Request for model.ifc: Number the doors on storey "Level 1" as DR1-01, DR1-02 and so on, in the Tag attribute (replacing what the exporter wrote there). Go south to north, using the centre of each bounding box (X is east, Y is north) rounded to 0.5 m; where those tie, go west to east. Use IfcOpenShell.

First a look at what the model holds.

```python
import ifcopenshell
import ifcopenshell.util.element
import ifcopenshell.util.placement

model = ifcopenshell.open("model.ifc")
print(model.schema)
storey = next(s for s in model.by_type("IfcBuildingStorey") if s.Name == "Level 1")
doors = [e for e in ifcopenshell.util.element.get_decomposition(storey) if e.is_a("IfcDoor")]
for e in sorted(doors, key=lambda e: e.id()):
    origin = ifcopenshell.util.placement.get_local_placement(e.ObjectPlacement)[:3, 3]
    print(e.id(), e.Tag, e.Name, origin.round(2) + 0.0, sep=" | ")
```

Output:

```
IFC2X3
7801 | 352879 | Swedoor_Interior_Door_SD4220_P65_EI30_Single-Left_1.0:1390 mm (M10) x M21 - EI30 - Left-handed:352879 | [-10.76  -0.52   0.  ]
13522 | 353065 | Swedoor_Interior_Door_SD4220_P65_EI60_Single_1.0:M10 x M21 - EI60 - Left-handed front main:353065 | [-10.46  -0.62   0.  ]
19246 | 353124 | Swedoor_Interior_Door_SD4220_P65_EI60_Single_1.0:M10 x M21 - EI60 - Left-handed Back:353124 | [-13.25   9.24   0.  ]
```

```python
import ifcopenshell
import ifcopenshell.geom
import ifcopenshell.util.element
import ifcopenshell.util.shape

model = ifcopenshell.open("model.ifc")
settings = ifcopenshell.geom.settings()
settings.set("use-world-coords", True)


def centre(element):
    shape = ifcopenshell.geom.create_shape(settings, element)
    return ifcopenshell.util.shape.get_bbox_centroid(shape.geometry)


storey = next(s for s in model.by_type("IfcBuildingStorey") if s.Name == "Level 1")
doors = [e for e in ifcopenshell.util.element.get_decomposition(storey) if e.is_a("IfcDoor")]

# Insertion points can sit at a corner or the storey origin, so sort by the geometry (in metres).
centres = {e: centre(e) for e in doors}
doors.sort(key=lambda e: (round(centres[e][1] / 0.5), centres[e][0]))

for i, e in enumerate(doors, start=1):
    number = f"DR1-{i:02d}"
    e.Tag = number
    print(e.id(), number)

model.write("model-out.ifc")
```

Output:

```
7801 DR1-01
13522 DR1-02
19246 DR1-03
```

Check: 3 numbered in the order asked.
